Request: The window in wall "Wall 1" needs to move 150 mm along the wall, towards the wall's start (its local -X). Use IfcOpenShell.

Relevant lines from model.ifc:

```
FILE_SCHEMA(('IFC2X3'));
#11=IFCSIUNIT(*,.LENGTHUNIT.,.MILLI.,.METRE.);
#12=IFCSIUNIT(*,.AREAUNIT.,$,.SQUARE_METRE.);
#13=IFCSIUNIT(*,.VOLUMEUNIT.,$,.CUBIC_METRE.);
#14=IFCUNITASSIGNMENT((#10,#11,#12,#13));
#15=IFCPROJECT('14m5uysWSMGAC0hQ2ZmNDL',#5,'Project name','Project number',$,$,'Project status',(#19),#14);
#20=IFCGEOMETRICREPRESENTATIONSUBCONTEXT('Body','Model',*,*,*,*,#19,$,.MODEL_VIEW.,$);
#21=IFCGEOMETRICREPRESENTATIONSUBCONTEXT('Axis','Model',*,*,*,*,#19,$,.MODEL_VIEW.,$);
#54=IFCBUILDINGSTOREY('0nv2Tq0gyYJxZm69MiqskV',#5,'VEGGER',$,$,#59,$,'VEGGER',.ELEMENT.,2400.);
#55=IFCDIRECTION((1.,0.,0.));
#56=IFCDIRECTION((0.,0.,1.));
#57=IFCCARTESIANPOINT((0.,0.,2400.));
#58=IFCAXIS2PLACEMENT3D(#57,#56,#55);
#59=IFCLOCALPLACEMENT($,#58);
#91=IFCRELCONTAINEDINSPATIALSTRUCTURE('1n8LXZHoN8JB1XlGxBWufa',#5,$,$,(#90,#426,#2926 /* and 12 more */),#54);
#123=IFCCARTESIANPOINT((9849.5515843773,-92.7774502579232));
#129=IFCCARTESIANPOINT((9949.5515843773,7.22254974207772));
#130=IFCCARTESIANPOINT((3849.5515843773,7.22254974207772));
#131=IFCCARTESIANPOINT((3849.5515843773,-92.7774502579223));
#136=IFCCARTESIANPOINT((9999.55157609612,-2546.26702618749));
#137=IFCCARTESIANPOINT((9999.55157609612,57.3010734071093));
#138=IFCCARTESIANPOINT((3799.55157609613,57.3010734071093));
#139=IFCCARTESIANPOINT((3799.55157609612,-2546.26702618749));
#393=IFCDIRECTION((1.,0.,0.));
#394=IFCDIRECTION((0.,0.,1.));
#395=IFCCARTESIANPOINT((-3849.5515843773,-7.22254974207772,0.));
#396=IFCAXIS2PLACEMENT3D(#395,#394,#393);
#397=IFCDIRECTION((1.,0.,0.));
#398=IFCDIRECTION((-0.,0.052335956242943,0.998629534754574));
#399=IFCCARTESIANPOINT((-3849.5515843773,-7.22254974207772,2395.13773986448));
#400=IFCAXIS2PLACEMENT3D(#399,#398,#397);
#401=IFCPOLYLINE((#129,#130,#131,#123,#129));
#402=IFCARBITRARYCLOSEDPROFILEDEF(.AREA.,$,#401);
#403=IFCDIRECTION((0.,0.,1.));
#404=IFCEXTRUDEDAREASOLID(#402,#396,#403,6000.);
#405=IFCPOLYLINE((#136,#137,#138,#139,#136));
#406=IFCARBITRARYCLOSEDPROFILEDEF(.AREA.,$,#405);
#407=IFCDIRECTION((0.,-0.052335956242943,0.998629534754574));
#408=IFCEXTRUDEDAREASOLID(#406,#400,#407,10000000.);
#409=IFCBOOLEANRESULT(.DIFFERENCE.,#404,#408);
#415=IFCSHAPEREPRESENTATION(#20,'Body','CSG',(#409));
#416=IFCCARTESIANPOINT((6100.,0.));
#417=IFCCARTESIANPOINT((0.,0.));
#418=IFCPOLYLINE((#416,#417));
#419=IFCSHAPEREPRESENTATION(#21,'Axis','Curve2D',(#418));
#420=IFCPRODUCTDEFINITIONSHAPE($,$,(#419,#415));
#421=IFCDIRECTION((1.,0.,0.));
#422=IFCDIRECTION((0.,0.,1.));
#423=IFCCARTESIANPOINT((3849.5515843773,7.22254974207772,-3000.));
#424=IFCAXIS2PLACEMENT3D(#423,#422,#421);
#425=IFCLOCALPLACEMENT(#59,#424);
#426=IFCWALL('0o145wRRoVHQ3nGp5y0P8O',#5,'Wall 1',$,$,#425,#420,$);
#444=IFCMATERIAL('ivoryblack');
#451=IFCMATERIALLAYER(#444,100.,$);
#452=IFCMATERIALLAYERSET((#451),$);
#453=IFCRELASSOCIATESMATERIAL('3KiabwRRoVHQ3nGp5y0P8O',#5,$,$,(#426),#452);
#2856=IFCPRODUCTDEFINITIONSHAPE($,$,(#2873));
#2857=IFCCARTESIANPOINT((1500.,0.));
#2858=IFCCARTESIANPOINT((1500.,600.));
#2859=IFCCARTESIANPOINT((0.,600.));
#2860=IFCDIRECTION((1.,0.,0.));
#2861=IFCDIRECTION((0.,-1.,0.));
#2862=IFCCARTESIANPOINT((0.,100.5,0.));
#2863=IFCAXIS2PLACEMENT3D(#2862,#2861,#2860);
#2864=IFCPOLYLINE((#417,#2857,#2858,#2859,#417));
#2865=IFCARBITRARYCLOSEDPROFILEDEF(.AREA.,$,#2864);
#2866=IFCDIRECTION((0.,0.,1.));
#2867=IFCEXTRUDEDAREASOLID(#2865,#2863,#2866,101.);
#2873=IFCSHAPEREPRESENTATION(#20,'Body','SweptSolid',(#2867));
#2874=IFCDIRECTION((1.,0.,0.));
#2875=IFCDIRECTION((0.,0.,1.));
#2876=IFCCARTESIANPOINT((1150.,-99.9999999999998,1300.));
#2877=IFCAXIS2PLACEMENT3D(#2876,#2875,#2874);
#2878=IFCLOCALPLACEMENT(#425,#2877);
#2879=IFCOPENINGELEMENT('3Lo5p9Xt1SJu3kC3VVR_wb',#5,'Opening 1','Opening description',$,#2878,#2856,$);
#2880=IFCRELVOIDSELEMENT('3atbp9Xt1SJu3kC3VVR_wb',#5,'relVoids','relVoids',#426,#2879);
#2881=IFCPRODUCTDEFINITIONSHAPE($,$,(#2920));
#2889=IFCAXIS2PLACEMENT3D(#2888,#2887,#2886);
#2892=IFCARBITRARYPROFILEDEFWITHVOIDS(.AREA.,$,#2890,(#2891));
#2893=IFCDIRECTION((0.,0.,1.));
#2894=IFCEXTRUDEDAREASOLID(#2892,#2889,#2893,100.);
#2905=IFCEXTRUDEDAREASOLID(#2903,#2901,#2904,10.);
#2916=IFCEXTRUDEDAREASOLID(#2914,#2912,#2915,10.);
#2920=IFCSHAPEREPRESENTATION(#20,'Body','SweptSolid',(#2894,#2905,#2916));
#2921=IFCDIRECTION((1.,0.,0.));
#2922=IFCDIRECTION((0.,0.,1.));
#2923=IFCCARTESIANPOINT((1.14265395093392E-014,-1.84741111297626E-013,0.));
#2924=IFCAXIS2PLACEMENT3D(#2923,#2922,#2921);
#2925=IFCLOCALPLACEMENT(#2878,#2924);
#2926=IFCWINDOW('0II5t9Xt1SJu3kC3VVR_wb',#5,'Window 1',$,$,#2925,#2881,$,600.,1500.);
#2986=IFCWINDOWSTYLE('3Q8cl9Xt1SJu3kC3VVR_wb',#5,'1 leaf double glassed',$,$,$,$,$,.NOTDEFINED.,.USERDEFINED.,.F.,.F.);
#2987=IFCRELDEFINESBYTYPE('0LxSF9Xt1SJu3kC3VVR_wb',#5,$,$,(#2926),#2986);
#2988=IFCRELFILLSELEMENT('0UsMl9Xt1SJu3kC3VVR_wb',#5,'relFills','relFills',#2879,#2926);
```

```python
import ifcopenshell
import ifcopenshell.api.geometry
import ifcopenshell.util.placement

model = ifcopenshell.open("model.ifc")

window = model.by_id(2926)
opening = window.FillsVoids[0].RelatingOpeningElement
wall = opening.VoidsElements[0].RelatingBuildingElement

wall_matrix = ifcopenshell.util.placement.get_local_placement(wall.ObjectPlacement)
shift = wall_matrix[:3, 0] * -150.0
before = ifcopenshell.util.placement.get_local_placement(window.ObjectPlacement)[:3, 3].copy()

# The window is placed relative to its opening, so it follows when the opening moves.
matrix = ifcopenshell.util.placement.get_local_placement(opening.ObjectPlacement)
matrix[:3, 3] += shift
ifcopenshell.api.geometry.edit_object_placement(
    model, product=opening, matrix=matrix, is_si=False, should_transform_children=True
)

after = ifcopenshell.util.placement.get_local_placement(window.ObjectPlacement)[:3, 3]
print("window moved by", (after - before).round(3) + 0.0)

model.write("model_rev.ifc")
```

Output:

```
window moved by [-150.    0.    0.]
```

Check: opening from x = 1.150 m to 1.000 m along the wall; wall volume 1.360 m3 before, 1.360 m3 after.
